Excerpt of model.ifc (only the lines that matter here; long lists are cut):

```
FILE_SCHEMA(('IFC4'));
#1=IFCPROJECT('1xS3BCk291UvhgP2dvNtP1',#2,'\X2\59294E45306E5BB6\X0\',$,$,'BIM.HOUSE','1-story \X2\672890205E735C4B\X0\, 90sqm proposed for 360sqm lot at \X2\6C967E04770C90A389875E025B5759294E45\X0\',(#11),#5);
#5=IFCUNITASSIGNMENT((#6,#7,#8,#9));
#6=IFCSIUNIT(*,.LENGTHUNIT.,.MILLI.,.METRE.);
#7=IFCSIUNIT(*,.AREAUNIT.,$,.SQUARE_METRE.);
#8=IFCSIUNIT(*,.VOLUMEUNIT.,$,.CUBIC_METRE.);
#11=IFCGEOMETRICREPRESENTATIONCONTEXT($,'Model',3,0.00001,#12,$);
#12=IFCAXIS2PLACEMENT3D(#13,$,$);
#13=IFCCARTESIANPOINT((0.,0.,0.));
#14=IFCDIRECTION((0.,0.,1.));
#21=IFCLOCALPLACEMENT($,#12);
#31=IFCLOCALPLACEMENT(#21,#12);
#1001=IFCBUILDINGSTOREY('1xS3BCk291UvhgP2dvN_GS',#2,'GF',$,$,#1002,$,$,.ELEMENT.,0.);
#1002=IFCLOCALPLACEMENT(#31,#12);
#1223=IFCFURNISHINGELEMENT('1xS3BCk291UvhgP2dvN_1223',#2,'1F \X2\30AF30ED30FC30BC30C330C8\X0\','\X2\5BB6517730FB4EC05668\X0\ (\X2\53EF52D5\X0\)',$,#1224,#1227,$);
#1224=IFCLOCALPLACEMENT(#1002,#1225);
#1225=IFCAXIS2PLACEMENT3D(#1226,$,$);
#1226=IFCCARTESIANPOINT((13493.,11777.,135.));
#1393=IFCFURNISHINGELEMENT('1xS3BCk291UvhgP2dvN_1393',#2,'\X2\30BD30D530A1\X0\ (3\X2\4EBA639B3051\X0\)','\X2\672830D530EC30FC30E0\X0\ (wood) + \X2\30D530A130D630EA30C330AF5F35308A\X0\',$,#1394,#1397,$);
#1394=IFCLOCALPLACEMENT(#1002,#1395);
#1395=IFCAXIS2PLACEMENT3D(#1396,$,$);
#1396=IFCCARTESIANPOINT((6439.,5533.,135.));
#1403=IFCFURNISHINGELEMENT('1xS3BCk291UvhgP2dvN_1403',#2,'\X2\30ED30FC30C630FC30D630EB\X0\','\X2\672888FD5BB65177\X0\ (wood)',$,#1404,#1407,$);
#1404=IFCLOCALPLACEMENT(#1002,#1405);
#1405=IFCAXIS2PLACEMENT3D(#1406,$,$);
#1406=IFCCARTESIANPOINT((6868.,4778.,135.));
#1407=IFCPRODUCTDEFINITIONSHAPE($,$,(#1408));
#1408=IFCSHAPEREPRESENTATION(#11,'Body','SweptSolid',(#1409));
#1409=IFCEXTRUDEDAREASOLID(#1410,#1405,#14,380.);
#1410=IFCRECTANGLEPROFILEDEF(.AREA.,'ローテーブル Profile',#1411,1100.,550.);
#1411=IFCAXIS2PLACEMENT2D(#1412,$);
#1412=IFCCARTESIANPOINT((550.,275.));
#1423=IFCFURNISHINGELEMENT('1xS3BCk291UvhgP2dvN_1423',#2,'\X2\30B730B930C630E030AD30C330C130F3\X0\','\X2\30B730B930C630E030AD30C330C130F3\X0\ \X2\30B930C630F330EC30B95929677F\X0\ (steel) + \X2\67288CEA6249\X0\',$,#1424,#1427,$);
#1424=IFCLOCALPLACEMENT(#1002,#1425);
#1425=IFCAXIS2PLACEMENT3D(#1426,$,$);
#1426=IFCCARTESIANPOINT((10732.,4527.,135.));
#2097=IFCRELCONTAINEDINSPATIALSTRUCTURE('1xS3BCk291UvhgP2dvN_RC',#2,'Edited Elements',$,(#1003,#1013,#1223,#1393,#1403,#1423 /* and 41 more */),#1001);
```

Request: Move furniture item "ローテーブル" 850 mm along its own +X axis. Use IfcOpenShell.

```python
import ifcopenshell
import ifcopenshell.api.geometry
import ifcopenshell.util.placement

model = ifcopenshell.open("model.ifc")

item = model.by_guid("1xS3BCk291UvhgP2dvN_1403")
matrix = ifcopenshell.util.placement.get_local_placement(item.ObjectPlacement)
matrix[:3, 3] += matrix[:3, 0] * 850.0
ifcopenshell.api.geometry.edit_object_placement(model, product=item, matrix=matrix, is_si=False)

print(ifcopenshell.util.placement.get_local_placement(item.ObjectPlacement).round(3) + 0.0)

model.write("model_v2.ifc")
```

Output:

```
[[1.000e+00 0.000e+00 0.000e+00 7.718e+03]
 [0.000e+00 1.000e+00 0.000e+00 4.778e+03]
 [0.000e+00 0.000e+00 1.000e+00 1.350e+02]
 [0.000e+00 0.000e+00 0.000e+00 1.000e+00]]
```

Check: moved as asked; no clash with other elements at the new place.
